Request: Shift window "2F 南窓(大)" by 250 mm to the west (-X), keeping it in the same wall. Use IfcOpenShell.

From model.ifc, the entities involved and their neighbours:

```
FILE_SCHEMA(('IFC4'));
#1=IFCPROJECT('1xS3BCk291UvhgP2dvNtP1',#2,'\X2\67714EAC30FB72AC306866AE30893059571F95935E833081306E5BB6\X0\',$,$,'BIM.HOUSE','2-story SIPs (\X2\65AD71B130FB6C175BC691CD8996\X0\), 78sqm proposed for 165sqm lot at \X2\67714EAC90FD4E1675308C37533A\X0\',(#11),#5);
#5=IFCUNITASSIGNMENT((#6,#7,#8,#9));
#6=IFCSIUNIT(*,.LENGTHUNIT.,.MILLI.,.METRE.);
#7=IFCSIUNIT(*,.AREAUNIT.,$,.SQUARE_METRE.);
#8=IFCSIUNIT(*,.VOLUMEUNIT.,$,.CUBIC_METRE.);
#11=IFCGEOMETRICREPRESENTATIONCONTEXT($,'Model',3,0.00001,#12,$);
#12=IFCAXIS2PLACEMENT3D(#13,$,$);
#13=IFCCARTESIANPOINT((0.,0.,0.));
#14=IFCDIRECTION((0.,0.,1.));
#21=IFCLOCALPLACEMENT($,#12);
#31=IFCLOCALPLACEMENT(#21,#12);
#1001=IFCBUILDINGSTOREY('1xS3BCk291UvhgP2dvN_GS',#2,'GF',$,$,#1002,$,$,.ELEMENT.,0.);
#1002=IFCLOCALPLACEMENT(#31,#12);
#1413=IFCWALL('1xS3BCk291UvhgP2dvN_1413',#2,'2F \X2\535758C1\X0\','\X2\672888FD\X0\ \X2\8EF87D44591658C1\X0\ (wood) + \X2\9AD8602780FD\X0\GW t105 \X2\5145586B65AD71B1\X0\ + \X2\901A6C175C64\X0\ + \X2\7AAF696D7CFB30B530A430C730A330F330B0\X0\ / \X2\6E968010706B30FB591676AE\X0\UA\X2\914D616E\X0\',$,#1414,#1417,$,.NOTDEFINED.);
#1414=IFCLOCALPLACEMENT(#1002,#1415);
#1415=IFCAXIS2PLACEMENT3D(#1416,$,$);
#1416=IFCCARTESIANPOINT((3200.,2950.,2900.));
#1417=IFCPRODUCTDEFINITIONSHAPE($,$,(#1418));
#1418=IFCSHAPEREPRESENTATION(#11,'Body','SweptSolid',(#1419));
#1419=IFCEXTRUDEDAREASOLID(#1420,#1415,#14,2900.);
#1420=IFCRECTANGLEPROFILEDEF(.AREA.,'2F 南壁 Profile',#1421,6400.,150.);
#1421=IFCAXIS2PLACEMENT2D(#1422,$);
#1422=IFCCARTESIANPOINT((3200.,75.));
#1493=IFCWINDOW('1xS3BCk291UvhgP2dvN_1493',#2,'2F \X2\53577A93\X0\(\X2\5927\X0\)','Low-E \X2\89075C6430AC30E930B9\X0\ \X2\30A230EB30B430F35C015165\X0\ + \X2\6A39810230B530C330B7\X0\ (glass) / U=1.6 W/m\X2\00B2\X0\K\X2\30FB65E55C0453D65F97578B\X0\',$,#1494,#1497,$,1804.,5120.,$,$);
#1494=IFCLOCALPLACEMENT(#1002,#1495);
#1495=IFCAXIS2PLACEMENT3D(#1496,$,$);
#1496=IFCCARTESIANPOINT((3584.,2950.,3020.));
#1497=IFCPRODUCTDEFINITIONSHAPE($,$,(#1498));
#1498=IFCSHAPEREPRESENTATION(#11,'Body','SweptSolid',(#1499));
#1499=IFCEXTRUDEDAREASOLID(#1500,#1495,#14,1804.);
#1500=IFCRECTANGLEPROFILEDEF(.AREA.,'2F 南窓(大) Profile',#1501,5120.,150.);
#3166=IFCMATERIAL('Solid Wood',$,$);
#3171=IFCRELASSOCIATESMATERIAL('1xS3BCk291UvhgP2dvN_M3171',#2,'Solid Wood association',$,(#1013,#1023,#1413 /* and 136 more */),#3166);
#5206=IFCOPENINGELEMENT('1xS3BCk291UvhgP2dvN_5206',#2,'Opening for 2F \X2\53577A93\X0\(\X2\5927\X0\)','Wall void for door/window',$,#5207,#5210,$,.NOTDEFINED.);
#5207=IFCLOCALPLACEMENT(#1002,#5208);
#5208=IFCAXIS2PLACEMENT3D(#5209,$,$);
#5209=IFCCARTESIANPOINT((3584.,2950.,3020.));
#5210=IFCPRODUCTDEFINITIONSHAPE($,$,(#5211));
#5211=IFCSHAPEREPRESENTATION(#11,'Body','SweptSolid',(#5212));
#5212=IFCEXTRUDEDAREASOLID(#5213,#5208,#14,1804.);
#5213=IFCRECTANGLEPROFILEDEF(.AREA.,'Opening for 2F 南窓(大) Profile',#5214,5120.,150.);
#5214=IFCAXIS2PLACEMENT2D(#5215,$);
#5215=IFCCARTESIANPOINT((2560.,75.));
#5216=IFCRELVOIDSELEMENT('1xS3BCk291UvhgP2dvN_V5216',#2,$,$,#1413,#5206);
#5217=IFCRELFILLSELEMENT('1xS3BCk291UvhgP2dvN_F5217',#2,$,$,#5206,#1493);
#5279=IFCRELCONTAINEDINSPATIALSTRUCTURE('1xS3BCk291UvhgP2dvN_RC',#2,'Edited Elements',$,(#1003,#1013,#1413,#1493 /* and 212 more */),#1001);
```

```python
import ifcopenshell
import ifcopenshell.api.geometry
import ifcopenshell.util.placement
import ifcopenshell.util.unit

model = ifcopenshell.open("model.ifc")
unit_scale = ifcopenshell.util.unit.calculate_unit_scale(model)

window = model.by_guid("1xS3BCk291UvhgP2dvN_1493")
opening = window.FillsVoids[0].RelatingOpeningElement
wall = opening.VoidsElements[0].RelatingBuildingElement

wall_matrix = ifcopenshell.util.placement.get_local_placement(wall.ObjectPlacement)
shift = wall_matrix[:3, 0] * -0.25 / unit_scale
before = ifcopenshell.util.placement.get_local_placement(window.ObjectPlacement)[:3, 3].copy()

# The window is not placed relative to its opening, so move both.
for product in (opening, window):
    matrix = ifcopenshell.util.placement.get_local_placement(product.ObjectPlacement)
    matrix[:3, 3] += shift
    ifcopenshell.api.geometry.edit_object_placement(model, product=product, matrix=matrix, is_si=False)

after = ifcopenshell.util.placement.get_local_placement(window.ObjectPlacement)[:3, 3]
print("window moved by", (after - before).round(3) + 0.0)

model.write("model_rev.ifc")
```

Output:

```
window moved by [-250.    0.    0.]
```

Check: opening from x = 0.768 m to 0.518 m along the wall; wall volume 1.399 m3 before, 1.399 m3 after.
